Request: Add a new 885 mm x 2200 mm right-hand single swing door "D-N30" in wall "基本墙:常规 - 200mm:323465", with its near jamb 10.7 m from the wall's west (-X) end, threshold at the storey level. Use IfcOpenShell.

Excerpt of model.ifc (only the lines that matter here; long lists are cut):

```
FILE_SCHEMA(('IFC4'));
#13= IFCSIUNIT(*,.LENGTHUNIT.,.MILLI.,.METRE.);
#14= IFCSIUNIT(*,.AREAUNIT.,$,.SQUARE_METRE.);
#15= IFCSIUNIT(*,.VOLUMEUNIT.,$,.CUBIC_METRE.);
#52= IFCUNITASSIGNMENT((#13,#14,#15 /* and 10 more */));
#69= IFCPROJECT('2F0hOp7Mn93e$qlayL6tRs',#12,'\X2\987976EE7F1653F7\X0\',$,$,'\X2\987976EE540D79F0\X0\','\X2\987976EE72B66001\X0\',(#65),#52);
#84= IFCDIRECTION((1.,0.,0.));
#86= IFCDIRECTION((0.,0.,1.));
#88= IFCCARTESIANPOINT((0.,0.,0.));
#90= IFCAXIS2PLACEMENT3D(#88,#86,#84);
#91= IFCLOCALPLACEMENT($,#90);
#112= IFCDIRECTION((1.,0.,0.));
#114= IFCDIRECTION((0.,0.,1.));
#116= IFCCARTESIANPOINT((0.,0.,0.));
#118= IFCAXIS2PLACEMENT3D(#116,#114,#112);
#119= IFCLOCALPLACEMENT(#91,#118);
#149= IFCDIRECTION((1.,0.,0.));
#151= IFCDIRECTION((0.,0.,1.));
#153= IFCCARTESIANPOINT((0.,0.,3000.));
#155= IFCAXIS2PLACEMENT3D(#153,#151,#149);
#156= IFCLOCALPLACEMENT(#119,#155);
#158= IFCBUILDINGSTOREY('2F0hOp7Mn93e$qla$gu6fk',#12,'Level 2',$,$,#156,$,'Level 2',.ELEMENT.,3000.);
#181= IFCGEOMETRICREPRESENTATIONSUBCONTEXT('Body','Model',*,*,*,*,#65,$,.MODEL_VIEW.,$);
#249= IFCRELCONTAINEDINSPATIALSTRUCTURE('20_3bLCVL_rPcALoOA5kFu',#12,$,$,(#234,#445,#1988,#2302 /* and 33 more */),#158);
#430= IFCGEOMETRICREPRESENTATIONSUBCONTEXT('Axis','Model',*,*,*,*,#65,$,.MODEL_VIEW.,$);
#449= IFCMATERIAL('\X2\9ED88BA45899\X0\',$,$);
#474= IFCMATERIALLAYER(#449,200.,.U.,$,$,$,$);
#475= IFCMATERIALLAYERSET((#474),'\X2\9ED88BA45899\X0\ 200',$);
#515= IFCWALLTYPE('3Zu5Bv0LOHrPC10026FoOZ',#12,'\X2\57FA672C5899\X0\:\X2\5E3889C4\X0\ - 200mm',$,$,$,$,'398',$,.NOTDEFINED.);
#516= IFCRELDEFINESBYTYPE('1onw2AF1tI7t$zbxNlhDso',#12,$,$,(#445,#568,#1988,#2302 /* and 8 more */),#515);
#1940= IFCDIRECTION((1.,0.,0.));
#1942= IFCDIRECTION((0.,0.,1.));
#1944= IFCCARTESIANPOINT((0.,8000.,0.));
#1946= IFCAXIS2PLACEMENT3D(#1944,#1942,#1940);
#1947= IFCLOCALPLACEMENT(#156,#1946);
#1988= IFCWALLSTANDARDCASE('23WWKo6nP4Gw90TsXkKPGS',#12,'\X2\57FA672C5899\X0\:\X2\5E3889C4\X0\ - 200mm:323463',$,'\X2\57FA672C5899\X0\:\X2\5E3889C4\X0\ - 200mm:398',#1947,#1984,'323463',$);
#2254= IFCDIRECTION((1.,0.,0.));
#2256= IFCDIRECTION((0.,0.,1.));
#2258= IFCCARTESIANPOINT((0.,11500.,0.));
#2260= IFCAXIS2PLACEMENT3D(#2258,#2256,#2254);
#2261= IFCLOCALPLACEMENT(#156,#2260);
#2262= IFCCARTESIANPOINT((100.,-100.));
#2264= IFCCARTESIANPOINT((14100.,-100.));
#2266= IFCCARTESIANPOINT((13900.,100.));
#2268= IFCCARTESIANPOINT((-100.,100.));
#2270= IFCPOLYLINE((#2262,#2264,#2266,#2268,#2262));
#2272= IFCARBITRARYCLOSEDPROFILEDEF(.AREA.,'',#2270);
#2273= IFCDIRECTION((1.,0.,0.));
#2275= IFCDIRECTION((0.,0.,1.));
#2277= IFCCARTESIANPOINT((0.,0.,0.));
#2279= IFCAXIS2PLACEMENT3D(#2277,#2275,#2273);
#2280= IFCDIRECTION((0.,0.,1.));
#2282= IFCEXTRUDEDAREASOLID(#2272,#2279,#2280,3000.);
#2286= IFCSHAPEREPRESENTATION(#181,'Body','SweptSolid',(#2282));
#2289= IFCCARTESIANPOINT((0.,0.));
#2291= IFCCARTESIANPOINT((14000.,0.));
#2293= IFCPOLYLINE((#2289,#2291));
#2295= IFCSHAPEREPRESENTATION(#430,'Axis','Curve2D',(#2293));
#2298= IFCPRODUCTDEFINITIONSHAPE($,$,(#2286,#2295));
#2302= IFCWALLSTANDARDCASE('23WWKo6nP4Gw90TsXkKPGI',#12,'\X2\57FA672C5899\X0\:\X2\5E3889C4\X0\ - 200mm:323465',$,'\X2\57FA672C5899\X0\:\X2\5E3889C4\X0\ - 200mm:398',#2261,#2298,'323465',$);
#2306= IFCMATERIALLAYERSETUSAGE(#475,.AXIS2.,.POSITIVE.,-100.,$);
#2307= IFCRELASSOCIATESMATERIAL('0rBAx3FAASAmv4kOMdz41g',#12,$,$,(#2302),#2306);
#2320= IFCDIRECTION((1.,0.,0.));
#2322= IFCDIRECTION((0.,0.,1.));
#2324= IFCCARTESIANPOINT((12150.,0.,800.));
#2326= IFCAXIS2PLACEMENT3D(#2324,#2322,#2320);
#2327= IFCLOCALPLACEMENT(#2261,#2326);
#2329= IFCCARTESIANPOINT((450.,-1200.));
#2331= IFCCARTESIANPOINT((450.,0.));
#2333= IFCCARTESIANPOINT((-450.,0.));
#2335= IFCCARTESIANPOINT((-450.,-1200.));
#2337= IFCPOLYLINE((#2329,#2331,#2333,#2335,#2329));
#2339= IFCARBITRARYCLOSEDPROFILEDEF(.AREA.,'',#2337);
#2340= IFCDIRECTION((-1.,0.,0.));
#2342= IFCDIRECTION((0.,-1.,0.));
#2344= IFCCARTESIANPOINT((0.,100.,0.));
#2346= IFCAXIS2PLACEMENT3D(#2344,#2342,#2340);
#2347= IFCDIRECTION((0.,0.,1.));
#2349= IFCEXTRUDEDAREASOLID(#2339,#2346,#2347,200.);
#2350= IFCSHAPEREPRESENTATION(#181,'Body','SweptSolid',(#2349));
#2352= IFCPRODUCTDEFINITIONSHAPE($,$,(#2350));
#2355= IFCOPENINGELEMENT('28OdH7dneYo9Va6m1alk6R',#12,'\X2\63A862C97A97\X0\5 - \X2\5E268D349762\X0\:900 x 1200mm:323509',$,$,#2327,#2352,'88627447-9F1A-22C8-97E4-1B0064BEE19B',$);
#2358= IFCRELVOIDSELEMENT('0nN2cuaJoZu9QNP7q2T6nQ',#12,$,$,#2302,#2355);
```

```python
import numpy as np
import ifcopenshell
import ifcopenshell.api.feature
import ifcopenshell.api.geometry
import ifcopenshell.api.root
import ifcopenshell.api.spatial
import ifcopenshell.geom
import ifcopenshell.util.element
import ifcopenshell.util.placement
import ifcopenshell.util.representation
import ifcopenshell.util.shape
import ifcopenshell.util.unit

model = ifcopenshell.open("model.ifc")
unit_scale = ifcopenshell.util.unit.calculate_unit_scale(model)
settings = ifcopenshell.geom.settings()


def volume(element):
    """Net volume in cubic metres, openings subtracted."""
    shape = ifcopenshell.geom.create_shape(settings, element)
    return ifcopenshell.util.shape.get_volume(shape.geometry)


wall = model.by_id(2302)
storey = ifcopenshell.util.element.get_container(wall, ifc_class="IfcBuildingStorey")
context = ifcopenshell.util.representation.get_context(model, "Model", "Body", "MODEL_VIEW")
before = volume(wall)

width, height, from_end, sill = 0.885, 2.2, 10.7, 0.0  # metres

# The wall runs along its own X axis, and the end named is its -X end.
wall_shape = ifcopenshell.geom.create_shape(settings, wall)
x, y, z = ifcopenshell.util.shape.get_vertices(wall_shape.geometry).T
start = x.min() + from_end
face, thickness = float(y.min()), float(y.max() - y.min())
wall_matrix = ifcopenshell.util.placement.get_local_placement(wall.ObjectPlacement)
level = ifcopenshell.util.placement.get_local_placement(storey.ObjectPlacement)[2, 3]


def in_wall(x, y):
    """Placement at x, y metres in the wall's axes, at sill height."""
    matrix = wall_matrix.copy()
    matrix[:, 3] = wall_matrix @ np.array([x / unit_scale, y / unit_scale, 0.0, 1.0])
    matrix[2, 3] = level + sill / unit_scale
    return matrix


# Opening: a box that overshoots both wall faces by 50 mm.
opening = ifcopenshell.api.root.create_entity(model, ifc_class="IfcOpeningElement", predefined_type="OPENING")
box = ifcopenshell.api.geometry.add_wall_representation(
    model, context=context, length=width, height=height, thickness=thickness + 0.1
)
ifcopenshell.api.geometry.assign_representation(model, product=opening, representation=box)
ifcopenshell.api.geometry.edit_object_placement(model, product=opening, matrix=in_wall(start, face - 0.05), is_si=False)
ifcopenshell.api.feature.add_feature(model, feature=opening, element=wall)

door = ifcopenshell.api.root.create_entity(model, ifc_class="IfcDoor", name="D-N30", predefined_type="DOOR")
door.OverallWidth, door.OverallHeight = width / unit_scale, height / unit_scale
door.OperationType = "SINGLE_SWING_RIGHT"
body = ifcopenshell.api.geometry.add_door_representation(
    model,
    context=context,
    overall_width=door.OverallWidth,
    overall_height=door.OverallHeight,
    operation_type="SINGLE_SWING_RIGHT",
    lining_properties={"LiningDepth": thickness / unit_scale, "ThresholdDepth": thickness / unit_scale},
)
ifcopenshell.api.geometry.assign_representation(model, product=door, representation=body)
ifcopenshell.api.spatial.assign_container(model, products=[door], relating_structure=storey)
ifcopenshell.api.feature.add_filling(model, opening=opening, element=door)

# The lining spans the wall, so the door starts at the wall face.
ifcopenshell.api.geometry.edit_object_placement(model, product=door, matrix=in_wall(start, face), is_si=False)

after = volume(wall)

print(f"wall volume {before:.3f} -> {after:.3f} m3")

model.write("model_rev.ifc")
```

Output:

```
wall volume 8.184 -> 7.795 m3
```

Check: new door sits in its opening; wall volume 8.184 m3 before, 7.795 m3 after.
